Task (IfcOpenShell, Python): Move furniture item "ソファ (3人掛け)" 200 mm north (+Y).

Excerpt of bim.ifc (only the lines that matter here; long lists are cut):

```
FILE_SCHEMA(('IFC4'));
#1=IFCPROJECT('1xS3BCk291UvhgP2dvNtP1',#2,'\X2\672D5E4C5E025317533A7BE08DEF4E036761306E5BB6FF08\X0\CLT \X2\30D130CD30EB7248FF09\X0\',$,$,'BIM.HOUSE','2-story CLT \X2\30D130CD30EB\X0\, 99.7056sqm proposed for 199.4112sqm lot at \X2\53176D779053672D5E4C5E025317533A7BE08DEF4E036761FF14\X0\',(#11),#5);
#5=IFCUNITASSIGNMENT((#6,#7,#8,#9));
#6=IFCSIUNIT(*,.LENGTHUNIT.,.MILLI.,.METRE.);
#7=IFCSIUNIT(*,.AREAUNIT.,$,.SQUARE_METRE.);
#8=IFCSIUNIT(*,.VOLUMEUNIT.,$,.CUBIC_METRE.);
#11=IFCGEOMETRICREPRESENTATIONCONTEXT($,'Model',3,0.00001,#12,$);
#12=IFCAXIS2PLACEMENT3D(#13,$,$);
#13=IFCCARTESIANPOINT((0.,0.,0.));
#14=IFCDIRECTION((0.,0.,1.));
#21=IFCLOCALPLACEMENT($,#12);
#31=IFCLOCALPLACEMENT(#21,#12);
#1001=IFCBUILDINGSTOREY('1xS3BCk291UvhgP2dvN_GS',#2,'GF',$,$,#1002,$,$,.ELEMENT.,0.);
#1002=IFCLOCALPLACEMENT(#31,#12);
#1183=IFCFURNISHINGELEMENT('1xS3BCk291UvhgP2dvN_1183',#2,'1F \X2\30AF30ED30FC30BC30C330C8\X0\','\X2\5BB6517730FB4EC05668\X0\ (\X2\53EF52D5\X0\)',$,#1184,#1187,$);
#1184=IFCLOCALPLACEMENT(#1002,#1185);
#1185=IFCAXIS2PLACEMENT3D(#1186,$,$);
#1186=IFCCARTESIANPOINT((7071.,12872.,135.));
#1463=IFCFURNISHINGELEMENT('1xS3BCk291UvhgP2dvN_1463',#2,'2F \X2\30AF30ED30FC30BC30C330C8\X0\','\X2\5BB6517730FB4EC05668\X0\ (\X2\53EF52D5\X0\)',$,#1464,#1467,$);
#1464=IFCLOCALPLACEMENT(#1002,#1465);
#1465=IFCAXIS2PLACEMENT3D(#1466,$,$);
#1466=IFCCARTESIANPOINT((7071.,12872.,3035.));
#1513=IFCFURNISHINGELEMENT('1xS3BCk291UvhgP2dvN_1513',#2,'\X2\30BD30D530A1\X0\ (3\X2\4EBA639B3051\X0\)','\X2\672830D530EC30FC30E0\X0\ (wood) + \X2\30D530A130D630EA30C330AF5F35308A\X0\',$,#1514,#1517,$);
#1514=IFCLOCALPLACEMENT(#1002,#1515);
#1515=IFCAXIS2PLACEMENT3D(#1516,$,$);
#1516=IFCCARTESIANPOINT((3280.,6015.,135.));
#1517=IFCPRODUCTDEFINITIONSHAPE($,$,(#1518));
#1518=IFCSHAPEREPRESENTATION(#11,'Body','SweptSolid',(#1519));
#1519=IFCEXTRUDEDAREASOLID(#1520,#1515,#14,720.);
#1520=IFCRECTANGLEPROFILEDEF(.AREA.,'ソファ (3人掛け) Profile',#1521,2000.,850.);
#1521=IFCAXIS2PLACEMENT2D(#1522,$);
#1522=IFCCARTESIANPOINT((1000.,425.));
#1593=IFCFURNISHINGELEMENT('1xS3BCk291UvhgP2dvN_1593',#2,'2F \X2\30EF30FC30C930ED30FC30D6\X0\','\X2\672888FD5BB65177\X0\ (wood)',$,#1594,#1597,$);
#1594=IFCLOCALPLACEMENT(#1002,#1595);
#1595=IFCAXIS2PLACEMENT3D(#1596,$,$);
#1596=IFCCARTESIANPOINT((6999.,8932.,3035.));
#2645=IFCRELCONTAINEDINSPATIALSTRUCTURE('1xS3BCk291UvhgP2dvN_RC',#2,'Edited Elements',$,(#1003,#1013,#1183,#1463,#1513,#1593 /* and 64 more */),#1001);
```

```python
import ifcopenshell
import ifcopenshell.api.geometry
import ifcopenshell.util.placement
import ifcopenshell.util.unit

model = ifcopenshell.open("bim.ifc")
unit_scale = ifcopenshell.util.unit.calculate_unit_scale(model)

item = model.by_id(1513)
matrix = ifcopenshell.util.placement.get_local_placement(item.ObjectPlacement)
matrix[1, 3] += 0.2 / unit_scale
ifcopenshell.api.geometry.edit_object_placement(model, product=item, matrix=matrix, is_si=False)

print(ifcopenshell.util.placement.get_local_placement(item.ObjectPlacement).round(3) + 0.0)

model.write("bim_updated.ifc")
```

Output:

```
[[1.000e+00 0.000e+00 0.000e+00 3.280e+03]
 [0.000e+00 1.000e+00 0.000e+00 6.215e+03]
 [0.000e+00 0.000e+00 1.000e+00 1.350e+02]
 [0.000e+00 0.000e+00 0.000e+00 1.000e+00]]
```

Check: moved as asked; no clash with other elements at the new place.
